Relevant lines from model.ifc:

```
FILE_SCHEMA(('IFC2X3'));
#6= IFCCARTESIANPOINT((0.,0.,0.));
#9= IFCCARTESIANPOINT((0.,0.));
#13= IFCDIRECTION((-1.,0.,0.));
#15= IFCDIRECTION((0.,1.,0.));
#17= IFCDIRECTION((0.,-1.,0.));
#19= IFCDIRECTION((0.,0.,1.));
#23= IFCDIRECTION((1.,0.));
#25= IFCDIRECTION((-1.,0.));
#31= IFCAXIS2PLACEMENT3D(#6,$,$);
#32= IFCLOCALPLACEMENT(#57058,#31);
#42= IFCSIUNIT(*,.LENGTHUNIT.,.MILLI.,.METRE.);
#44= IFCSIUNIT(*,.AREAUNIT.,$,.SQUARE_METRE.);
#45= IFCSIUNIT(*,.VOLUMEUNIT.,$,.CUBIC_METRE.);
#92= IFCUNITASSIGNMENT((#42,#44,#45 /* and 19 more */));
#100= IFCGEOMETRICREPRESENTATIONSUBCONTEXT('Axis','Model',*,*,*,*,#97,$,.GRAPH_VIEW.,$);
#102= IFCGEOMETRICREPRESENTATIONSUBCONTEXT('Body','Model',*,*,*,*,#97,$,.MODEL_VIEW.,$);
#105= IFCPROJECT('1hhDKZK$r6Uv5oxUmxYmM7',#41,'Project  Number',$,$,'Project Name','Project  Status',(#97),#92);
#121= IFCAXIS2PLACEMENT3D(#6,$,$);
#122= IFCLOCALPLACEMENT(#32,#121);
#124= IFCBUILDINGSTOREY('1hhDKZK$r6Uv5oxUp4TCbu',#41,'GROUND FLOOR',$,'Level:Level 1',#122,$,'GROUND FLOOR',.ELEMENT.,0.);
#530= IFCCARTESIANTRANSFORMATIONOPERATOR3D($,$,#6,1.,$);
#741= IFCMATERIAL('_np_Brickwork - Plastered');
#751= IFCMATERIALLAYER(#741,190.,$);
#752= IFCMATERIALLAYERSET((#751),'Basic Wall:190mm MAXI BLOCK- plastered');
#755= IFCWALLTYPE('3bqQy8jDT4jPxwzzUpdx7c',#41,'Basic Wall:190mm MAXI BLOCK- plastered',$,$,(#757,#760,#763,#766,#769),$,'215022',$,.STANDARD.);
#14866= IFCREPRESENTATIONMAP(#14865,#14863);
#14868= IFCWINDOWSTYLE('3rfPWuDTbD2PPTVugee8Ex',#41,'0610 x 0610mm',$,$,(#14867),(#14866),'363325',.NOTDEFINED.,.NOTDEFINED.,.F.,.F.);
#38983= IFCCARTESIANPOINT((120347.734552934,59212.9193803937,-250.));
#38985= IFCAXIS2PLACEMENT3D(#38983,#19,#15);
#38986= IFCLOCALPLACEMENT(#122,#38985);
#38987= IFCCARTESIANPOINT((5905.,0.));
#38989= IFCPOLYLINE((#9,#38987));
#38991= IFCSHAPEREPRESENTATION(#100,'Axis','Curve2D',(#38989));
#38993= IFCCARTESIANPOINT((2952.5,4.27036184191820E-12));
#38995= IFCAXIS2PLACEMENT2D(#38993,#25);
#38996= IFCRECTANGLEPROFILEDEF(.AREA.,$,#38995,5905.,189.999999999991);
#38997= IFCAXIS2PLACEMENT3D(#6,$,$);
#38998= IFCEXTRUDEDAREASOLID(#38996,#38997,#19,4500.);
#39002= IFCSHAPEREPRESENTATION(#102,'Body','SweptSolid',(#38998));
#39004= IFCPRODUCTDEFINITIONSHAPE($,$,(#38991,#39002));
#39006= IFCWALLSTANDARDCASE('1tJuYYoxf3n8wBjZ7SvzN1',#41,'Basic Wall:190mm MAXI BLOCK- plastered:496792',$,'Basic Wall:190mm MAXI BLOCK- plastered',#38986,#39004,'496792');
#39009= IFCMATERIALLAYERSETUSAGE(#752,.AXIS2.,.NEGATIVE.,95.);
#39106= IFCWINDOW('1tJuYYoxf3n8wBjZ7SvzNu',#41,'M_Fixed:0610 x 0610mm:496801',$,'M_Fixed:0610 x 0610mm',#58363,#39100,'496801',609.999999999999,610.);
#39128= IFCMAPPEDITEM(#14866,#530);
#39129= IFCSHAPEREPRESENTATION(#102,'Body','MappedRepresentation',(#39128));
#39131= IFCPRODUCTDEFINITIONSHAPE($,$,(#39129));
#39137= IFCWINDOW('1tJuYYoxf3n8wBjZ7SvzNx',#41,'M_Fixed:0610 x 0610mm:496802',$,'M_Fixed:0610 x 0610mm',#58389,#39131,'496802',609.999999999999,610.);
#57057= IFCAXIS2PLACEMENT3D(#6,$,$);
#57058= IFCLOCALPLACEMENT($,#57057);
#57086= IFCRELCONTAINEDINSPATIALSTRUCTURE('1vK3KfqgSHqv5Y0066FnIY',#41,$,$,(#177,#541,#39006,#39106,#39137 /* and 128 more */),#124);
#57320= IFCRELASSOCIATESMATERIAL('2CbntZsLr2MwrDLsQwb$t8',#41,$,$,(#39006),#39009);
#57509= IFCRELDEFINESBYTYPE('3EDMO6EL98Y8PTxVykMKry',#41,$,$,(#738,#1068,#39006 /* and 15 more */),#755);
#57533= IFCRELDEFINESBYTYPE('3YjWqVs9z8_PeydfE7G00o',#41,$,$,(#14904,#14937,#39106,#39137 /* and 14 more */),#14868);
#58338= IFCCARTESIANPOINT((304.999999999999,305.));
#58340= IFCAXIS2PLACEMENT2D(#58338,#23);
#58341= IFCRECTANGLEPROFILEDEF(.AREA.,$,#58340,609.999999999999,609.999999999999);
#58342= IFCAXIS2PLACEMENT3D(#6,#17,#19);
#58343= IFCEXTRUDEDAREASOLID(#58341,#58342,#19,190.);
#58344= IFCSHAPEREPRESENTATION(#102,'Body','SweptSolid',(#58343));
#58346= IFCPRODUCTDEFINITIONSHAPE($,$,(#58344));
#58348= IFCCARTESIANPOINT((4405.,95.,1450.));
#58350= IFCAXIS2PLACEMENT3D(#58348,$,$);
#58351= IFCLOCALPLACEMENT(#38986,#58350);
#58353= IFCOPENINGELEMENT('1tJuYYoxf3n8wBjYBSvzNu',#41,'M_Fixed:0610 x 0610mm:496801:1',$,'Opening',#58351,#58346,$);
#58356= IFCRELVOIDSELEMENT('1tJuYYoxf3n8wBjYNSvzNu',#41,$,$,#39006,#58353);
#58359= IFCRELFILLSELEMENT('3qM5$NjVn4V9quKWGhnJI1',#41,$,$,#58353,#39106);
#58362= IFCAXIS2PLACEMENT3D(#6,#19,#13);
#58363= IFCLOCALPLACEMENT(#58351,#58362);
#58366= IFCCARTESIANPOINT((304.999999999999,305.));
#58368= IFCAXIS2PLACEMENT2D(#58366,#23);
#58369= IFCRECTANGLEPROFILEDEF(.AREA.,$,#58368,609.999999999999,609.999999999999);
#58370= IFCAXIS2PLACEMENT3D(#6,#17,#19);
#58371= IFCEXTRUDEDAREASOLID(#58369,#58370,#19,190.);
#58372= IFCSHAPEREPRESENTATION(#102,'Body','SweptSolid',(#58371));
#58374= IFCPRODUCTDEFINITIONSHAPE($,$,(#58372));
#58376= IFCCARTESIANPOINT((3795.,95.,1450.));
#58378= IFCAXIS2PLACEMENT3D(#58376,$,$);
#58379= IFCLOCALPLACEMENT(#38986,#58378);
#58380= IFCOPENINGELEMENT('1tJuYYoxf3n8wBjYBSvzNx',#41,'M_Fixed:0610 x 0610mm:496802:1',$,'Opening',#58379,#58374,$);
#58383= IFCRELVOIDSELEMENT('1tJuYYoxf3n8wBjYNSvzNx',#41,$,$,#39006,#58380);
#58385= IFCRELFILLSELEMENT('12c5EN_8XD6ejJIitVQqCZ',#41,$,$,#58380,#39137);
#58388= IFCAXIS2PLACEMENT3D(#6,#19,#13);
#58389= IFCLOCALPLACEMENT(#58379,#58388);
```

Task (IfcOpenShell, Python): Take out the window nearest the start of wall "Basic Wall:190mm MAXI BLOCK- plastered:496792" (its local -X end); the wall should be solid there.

```python
import ifcopenshell
import ifcopenshell.api.feature
import ifcopenshell.api.root
import ifcopenshell.geom
import ifcopenshell.util.shape

model = ifcopenshell.open("model.ifc")
settings = ifcopenshell.geom.settings()


def volume(element):
    """Net volume in cubic metres, openings subtracted."""
    shape = ifcopenshell.geom.create_shape(settings, element)
    return ifcopenshell.util.shape.get_volume(shape.geometry)


window = model.by_id(39137)
opening = window.FillsVoids[0].RelatingOpeningElement
wall = opening.VoidsElements[0].RelatingBuildingElement
before = volume(wall)

ifcopenshell.api.root.remove_product(model, product=window)
ifcopenshell.api.feature.remove_feature(model, feature=opening)

after = volume(wall)

print(f"wall volume {before:.3f} -> {after:.3f} m3")

model.write("model_edited.ifc")
```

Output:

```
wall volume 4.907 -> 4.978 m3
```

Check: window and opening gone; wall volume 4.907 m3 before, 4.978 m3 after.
